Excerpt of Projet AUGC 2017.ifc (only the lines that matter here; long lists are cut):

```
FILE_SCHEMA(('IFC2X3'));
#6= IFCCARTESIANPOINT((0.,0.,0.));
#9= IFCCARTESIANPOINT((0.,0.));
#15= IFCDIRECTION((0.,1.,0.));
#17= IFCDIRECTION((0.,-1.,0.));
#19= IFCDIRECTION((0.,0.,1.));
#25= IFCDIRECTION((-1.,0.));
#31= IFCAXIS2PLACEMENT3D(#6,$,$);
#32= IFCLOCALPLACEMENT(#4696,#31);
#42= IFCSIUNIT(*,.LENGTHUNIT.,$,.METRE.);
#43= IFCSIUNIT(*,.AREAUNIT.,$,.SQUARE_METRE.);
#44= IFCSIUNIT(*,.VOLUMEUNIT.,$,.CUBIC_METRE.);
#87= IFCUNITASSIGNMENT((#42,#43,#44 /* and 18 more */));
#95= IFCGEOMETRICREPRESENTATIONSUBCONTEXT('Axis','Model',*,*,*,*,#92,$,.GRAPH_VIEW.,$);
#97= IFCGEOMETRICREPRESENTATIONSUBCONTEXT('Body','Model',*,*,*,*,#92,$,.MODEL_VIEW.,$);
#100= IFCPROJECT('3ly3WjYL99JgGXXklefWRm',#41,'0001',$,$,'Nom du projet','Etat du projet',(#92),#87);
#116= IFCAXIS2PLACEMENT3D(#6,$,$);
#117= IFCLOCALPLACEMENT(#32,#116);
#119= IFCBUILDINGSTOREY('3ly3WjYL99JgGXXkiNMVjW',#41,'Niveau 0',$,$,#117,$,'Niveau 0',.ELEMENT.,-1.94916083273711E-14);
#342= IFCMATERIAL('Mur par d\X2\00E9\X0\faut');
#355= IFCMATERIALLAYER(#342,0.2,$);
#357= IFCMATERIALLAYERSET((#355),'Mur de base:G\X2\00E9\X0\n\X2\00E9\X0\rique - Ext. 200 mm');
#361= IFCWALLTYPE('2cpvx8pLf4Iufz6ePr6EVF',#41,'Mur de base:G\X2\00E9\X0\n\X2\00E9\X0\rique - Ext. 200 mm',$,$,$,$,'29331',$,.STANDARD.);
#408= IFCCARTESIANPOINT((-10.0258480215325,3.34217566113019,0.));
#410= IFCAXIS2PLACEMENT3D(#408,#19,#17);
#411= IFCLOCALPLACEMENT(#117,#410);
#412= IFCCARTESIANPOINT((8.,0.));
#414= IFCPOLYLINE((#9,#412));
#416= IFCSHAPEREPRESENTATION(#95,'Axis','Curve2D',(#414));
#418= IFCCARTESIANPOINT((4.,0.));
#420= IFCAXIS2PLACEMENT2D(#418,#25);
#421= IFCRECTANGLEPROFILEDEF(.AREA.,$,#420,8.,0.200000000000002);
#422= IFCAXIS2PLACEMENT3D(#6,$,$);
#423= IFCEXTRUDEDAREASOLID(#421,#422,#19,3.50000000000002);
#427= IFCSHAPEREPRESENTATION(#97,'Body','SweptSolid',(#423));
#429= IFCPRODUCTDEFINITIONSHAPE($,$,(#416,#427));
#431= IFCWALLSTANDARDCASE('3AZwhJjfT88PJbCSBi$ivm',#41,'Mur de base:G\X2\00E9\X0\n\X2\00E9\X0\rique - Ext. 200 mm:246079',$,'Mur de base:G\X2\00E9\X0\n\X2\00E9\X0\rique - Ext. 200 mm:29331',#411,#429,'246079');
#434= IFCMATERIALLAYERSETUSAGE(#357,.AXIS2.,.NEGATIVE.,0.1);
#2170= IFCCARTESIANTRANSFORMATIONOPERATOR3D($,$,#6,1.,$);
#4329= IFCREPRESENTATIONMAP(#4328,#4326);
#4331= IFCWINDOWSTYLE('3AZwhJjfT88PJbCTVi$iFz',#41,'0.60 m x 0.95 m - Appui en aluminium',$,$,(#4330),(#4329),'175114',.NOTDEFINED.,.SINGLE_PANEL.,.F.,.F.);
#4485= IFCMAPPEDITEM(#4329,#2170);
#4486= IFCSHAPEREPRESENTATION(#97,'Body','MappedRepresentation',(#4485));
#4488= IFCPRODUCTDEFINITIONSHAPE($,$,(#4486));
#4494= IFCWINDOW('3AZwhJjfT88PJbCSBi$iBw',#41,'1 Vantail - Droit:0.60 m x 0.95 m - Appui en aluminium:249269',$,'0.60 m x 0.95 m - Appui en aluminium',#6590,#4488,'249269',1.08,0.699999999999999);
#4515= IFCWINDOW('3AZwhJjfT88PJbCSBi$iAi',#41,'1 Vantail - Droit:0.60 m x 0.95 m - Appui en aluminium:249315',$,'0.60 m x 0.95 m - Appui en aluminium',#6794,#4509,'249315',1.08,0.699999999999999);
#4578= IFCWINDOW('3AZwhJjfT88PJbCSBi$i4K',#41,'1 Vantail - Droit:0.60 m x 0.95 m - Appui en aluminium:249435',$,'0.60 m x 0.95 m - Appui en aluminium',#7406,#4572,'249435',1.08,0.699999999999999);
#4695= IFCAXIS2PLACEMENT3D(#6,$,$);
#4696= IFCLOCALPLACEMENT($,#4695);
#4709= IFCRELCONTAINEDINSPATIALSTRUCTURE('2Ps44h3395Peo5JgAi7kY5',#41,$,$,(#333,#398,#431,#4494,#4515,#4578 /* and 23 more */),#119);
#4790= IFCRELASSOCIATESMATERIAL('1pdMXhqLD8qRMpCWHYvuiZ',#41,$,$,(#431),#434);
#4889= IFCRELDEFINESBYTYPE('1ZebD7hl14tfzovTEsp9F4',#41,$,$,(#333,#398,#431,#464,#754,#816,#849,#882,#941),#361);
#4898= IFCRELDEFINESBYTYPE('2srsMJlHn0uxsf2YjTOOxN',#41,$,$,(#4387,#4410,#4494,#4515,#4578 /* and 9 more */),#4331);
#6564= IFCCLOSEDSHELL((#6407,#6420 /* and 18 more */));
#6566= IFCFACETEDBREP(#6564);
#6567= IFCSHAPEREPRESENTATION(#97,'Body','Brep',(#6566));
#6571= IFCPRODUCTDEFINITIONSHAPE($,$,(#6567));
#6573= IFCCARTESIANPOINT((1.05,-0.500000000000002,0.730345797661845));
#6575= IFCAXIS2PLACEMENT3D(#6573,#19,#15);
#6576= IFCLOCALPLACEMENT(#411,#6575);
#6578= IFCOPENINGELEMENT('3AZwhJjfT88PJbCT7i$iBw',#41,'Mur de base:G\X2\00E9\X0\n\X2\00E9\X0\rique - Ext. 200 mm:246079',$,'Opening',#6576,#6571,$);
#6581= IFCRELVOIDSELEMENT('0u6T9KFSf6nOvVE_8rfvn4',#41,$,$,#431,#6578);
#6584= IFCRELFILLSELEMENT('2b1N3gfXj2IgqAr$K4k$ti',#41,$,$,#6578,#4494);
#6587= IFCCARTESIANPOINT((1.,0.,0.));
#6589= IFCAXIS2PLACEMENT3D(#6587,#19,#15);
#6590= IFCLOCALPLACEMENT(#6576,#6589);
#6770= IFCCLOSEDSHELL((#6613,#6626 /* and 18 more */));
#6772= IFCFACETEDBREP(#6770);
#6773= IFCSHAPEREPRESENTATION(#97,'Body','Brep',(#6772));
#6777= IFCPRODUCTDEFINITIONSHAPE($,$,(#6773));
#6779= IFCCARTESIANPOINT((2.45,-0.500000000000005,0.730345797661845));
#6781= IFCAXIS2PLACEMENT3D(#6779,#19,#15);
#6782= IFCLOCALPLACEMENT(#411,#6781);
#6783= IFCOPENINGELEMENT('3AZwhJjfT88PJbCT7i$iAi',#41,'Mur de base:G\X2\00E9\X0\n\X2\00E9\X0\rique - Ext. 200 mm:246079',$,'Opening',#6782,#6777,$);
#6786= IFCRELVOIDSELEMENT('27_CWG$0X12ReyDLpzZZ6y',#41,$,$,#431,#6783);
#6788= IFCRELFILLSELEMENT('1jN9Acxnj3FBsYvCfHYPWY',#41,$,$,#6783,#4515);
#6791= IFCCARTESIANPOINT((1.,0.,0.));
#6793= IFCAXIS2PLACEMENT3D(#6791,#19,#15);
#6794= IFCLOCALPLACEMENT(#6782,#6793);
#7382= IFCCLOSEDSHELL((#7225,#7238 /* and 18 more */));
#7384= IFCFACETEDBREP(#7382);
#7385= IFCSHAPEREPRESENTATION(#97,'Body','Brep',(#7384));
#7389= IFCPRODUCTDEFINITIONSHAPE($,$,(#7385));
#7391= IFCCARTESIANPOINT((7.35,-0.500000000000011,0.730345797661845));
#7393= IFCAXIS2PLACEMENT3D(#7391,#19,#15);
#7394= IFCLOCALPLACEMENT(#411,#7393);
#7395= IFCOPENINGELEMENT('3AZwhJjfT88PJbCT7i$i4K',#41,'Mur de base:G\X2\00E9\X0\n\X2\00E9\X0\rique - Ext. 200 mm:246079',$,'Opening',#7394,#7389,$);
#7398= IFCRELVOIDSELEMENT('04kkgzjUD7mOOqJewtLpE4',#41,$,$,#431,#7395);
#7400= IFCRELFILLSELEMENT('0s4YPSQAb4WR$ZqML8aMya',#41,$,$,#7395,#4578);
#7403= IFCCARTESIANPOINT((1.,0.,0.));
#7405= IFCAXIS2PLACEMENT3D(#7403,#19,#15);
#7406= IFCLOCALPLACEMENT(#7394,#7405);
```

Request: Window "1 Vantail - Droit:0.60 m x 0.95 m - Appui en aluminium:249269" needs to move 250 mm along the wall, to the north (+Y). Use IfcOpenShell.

```python
import ifcopenshell
import ifcopenshell.api.geometry
import ifcopenshell.util.placement
import ifcopenshell.util.unit

model = ifcopenshell.open("Projet AUGC 2017.ifc")
unit_scale = ifcopenshell.util.unit.calculate_unit_scale(model)

window = model.by_id(4494)
opening = window.FillsVoids[0].RelatingOpeningElement
wall = opening.VoidsElements[0].RelatingBuildingElement

wall_matrix = ifcopenshell.util.placement.get_local_placement(wall.ObjectPlacement)
shift = wall_matrix[:3, 0] * -0.25 / unit_scale
before = ifcopenshell.util.placement.get_local_placement(window.ObjectPlacement)[:3, 3].copy()

# The window is placed relative to its opening, so it follows when the opening moves.
matrix = ifcopenshell.util.placement.get_local_placement(opening.ObjectPlacement)
matrix[:3, 3] += shift
ifcopenshell.api.geometry.edit_object_placement(
    model, product=opening, matrix=matrix, is_si=False, should_transform_children=True
)

after = ifcopenshell.util.placement.get_local_placement(window.ObjectPlacement)[:3, 3]
print("window moved by", (after - before).round(3) + 0.0)

model.write("Projet AUGC 2017-out.ifc")
```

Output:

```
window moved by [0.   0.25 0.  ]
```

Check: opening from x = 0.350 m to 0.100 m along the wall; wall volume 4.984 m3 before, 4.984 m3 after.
